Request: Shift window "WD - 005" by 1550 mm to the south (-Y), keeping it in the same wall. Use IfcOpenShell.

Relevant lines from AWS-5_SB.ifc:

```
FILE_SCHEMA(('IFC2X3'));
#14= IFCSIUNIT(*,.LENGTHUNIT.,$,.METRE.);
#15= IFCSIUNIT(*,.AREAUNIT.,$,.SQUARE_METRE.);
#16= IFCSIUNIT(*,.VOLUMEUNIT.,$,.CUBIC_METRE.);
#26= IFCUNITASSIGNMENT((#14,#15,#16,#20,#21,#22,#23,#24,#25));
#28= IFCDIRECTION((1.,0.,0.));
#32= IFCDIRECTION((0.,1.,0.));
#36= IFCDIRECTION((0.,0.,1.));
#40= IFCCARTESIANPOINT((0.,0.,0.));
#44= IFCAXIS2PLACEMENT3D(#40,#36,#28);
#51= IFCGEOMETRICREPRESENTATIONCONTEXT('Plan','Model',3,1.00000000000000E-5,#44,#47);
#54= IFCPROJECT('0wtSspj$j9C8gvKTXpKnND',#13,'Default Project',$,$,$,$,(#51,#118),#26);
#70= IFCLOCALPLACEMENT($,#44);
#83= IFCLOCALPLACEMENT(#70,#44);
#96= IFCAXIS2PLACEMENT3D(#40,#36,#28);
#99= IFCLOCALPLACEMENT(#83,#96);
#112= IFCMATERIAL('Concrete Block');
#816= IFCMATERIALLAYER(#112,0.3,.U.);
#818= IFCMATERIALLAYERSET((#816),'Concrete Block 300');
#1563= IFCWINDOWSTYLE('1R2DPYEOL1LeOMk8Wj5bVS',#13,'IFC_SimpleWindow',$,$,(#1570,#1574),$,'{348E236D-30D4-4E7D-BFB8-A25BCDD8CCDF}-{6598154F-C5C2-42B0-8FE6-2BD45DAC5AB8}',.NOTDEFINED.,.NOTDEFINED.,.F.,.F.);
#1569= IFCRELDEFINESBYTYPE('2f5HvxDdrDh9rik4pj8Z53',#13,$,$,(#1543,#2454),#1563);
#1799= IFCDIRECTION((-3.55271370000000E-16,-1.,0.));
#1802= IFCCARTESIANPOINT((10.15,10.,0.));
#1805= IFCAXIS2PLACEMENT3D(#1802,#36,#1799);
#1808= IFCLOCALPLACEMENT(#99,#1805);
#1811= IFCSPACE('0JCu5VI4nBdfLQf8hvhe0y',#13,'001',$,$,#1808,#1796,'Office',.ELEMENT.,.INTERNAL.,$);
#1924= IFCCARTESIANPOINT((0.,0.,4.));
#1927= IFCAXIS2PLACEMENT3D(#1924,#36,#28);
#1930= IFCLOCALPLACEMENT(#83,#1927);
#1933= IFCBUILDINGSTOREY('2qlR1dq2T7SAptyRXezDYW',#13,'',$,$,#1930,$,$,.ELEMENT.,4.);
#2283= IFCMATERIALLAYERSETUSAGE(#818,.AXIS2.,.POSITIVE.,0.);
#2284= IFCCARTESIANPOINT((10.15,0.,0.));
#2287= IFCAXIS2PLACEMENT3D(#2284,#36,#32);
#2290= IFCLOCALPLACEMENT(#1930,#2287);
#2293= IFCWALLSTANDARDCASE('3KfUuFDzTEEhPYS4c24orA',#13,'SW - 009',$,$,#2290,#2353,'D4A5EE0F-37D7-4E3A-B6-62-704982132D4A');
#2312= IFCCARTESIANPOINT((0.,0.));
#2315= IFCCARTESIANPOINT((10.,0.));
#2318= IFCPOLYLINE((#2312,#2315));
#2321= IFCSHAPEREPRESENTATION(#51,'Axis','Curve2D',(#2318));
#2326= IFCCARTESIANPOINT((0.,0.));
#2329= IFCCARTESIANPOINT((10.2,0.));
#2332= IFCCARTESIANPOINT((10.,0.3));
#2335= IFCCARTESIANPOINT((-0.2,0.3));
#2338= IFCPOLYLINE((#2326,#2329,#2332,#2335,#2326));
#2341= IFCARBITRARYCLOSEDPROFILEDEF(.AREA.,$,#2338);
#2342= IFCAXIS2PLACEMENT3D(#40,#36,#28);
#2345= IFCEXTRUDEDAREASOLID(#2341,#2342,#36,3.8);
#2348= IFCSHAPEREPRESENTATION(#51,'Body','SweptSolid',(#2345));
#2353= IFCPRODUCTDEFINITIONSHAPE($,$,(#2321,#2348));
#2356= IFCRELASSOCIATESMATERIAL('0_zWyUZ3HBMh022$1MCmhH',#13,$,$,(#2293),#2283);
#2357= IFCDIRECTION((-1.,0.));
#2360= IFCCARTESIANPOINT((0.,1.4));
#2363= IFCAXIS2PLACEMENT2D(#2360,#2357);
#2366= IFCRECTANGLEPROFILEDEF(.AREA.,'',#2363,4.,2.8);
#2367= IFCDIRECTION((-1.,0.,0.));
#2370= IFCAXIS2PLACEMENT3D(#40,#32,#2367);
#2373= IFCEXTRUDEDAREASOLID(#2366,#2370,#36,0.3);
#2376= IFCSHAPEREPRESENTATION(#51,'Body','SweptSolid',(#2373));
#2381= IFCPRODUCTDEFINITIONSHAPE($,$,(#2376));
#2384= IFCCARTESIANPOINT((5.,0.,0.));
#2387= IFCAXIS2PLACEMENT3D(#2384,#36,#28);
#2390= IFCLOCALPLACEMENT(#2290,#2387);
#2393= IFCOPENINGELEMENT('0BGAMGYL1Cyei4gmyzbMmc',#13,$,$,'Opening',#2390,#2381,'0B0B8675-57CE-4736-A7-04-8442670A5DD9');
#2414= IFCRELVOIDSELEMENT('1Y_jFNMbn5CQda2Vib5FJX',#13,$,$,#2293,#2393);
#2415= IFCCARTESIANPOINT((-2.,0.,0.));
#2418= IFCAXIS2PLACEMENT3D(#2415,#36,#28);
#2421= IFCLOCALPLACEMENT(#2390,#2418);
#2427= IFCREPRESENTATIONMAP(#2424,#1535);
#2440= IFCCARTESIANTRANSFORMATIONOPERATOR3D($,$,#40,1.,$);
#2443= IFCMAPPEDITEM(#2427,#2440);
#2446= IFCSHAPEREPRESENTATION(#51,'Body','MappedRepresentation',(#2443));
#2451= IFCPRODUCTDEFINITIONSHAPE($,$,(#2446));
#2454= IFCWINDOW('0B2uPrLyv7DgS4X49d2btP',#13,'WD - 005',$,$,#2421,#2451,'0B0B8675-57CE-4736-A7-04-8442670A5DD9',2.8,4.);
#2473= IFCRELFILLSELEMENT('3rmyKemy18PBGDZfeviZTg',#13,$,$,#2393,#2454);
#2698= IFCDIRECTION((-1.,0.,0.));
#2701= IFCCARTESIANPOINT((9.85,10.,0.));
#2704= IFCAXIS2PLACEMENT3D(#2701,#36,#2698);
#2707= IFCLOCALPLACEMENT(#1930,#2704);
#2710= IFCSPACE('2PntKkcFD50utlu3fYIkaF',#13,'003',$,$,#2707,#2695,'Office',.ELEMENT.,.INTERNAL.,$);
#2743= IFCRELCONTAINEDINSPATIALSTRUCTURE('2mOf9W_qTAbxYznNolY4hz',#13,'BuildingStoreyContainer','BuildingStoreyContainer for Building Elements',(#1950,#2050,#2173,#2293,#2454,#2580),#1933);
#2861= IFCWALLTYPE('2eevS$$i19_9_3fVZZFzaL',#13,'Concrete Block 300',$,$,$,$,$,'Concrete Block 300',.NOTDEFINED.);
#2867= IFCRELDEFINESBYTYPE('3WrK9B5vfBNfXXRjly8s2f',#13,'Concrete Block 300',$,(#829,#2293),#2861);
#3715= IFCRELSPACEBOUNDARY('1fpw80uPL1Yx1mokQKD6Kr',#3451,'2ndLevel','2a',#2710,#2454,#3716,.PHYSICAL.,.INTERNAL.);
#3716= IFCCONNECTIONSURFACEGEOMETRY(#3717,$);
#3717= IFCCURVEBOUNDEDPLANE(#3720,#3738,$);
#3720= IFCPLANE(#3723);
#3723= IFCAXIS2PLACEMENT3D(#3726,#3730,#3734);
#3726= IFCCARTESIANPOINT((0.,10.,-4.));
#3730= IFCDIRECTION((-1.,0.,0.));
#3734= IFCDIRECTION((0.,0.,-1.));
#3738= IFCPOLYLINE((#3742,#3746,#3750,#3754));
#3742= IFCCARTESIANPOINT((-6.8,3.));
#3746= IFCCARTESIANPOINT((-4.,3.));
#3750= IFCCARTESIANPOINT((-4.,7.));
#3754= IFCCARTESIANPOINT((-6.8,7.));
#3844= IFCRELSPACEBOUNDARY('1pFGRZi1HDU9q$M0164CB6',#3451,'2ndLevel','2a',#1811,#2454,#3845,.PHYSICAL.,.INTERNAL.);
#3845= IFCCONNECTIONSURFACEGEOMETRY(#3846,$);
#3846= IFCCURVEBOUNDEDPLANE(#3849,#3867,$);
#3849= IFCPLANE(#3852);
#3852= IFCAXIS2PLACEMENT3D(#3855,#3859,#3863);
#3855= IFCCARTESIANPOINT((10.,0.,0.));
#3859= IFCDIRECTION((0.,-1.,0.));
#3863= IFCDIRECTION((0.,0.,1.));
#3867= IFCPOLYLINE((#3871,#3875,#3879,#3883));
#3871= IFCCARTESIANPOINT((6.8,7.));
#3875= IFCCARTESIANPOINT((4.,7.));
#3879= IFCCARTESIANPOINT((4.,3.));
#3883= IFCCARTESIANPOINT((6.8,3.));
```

```python
import numpy as np
import ifcopenshell
import ifcopenshell.api.geometry
import ifcopenshell.util.placement
import ifcopenshell.util.unit

model = ifcopenshell.open("AWS-5_SB.ifc")
unit_scale = ifcopenshell.util.unit.calculate_unit_scale(model)

window = model.by_guid("0B2uPrLyv7DgS4X49d2btP")
opening = window.FillsVoids[0].RelatingOpeningElement
wall = opening.VoidsElements[0].RelatingBuildingElement

wall_matrix = ifcopenshell.util.placement.get_local_placement(wall.ObjectPlacement)
shift = wall_matrix[:3, 0] * -1.55 / unit_scale
before = ifcopenshell.util.placement.get_local_placement(window.ObjectPlacement)[:3, 3].copy()

# The window is placed relative to its opening, so it follows when the opening moves.
matrix = ifcopenshell.util.placement.get_local_placement(opening.ObjectPlacement)
matrix[:3, 3] += shift
ifcopenshell.api.geometry.edit_object_placement(
    model, product=opening, matrix=matrix, is_si=False, should_transform_children=True
)

# Space boundary surfaces are stored in each space's coordinates; move them too.
for rel in window.ProvidesBoundaries:
    if not rel.ConnectionGeometry:
        continue
    surface = rel.ConnectionGeometry.SurfaceOnRelatingElement.BasisSurface
    space_matrix = ifcopenshell.util.placement.get_local_placement(rel.RelatingSpace.ObjectPlacement)
    point = np.array(surface.Position.Location.Coordinates) + space_matrix[:3, :3].T @ shift
    surface.Position = model.createIfcAxis2Placement3D(
        model.createIfcCartesianPoint(point.tolist()), surface.Position.Axis, surface.Position.RefDirection
    )

after = ifcopenshell.util.placement.get_local_placement(window.ObjectPlacement)[:3, 3]
print("window moved by", (after - before).round(3) + 0.0)

model.write("AWS-5_SB_rev.ifc")
```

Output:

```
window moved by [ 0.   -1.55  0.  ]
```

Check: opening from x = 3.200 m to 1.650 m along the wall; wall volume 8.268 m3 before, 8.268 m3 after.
